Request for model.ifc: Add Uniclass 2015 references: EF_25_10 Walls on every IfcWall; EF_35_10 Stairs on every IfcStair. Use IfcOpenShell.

First a look at what the model holds.

```python
import ifcopenshell

model = ifcopenshell.open("model.ifc")
print(model.schema)
print("classifications:", [c.Name for c in model.by_type("IfcClassification")])
for ifc_class in ("IfcDoor", "IfcRoof", "IfcStair", "IfcWall", "IfcWindow"):
    print(ifc_class, len(model.by_type(ifc_class)))
```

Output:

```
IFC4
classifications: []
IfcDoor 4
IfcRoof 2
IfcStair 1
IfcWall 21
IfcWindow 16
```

```python
import ifcopenshell
import ifcopenshell.api.classification

model = ifcopenshell.open("model.ifc")

system = ifcopenshell.api.classification.add_classification(model, classification="Uniclass 2015")

codes = {
    "IfcWall": ("EF_25_10", "Walls"),
    "IfcStair": ("EF_35_10", "Stairs"),
}
for ifc_class, (code, name) in codes.items():
    products = model.by_type(ifc_class)
    ifcopenshell.api.classification.add_reference(
        model, products=products, classification=system, identification=code, name=name
    )
    print(code, len(products))

model.write("model-out.ifc")
```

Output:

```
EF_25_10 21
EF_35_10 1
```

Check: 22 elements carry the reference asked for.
